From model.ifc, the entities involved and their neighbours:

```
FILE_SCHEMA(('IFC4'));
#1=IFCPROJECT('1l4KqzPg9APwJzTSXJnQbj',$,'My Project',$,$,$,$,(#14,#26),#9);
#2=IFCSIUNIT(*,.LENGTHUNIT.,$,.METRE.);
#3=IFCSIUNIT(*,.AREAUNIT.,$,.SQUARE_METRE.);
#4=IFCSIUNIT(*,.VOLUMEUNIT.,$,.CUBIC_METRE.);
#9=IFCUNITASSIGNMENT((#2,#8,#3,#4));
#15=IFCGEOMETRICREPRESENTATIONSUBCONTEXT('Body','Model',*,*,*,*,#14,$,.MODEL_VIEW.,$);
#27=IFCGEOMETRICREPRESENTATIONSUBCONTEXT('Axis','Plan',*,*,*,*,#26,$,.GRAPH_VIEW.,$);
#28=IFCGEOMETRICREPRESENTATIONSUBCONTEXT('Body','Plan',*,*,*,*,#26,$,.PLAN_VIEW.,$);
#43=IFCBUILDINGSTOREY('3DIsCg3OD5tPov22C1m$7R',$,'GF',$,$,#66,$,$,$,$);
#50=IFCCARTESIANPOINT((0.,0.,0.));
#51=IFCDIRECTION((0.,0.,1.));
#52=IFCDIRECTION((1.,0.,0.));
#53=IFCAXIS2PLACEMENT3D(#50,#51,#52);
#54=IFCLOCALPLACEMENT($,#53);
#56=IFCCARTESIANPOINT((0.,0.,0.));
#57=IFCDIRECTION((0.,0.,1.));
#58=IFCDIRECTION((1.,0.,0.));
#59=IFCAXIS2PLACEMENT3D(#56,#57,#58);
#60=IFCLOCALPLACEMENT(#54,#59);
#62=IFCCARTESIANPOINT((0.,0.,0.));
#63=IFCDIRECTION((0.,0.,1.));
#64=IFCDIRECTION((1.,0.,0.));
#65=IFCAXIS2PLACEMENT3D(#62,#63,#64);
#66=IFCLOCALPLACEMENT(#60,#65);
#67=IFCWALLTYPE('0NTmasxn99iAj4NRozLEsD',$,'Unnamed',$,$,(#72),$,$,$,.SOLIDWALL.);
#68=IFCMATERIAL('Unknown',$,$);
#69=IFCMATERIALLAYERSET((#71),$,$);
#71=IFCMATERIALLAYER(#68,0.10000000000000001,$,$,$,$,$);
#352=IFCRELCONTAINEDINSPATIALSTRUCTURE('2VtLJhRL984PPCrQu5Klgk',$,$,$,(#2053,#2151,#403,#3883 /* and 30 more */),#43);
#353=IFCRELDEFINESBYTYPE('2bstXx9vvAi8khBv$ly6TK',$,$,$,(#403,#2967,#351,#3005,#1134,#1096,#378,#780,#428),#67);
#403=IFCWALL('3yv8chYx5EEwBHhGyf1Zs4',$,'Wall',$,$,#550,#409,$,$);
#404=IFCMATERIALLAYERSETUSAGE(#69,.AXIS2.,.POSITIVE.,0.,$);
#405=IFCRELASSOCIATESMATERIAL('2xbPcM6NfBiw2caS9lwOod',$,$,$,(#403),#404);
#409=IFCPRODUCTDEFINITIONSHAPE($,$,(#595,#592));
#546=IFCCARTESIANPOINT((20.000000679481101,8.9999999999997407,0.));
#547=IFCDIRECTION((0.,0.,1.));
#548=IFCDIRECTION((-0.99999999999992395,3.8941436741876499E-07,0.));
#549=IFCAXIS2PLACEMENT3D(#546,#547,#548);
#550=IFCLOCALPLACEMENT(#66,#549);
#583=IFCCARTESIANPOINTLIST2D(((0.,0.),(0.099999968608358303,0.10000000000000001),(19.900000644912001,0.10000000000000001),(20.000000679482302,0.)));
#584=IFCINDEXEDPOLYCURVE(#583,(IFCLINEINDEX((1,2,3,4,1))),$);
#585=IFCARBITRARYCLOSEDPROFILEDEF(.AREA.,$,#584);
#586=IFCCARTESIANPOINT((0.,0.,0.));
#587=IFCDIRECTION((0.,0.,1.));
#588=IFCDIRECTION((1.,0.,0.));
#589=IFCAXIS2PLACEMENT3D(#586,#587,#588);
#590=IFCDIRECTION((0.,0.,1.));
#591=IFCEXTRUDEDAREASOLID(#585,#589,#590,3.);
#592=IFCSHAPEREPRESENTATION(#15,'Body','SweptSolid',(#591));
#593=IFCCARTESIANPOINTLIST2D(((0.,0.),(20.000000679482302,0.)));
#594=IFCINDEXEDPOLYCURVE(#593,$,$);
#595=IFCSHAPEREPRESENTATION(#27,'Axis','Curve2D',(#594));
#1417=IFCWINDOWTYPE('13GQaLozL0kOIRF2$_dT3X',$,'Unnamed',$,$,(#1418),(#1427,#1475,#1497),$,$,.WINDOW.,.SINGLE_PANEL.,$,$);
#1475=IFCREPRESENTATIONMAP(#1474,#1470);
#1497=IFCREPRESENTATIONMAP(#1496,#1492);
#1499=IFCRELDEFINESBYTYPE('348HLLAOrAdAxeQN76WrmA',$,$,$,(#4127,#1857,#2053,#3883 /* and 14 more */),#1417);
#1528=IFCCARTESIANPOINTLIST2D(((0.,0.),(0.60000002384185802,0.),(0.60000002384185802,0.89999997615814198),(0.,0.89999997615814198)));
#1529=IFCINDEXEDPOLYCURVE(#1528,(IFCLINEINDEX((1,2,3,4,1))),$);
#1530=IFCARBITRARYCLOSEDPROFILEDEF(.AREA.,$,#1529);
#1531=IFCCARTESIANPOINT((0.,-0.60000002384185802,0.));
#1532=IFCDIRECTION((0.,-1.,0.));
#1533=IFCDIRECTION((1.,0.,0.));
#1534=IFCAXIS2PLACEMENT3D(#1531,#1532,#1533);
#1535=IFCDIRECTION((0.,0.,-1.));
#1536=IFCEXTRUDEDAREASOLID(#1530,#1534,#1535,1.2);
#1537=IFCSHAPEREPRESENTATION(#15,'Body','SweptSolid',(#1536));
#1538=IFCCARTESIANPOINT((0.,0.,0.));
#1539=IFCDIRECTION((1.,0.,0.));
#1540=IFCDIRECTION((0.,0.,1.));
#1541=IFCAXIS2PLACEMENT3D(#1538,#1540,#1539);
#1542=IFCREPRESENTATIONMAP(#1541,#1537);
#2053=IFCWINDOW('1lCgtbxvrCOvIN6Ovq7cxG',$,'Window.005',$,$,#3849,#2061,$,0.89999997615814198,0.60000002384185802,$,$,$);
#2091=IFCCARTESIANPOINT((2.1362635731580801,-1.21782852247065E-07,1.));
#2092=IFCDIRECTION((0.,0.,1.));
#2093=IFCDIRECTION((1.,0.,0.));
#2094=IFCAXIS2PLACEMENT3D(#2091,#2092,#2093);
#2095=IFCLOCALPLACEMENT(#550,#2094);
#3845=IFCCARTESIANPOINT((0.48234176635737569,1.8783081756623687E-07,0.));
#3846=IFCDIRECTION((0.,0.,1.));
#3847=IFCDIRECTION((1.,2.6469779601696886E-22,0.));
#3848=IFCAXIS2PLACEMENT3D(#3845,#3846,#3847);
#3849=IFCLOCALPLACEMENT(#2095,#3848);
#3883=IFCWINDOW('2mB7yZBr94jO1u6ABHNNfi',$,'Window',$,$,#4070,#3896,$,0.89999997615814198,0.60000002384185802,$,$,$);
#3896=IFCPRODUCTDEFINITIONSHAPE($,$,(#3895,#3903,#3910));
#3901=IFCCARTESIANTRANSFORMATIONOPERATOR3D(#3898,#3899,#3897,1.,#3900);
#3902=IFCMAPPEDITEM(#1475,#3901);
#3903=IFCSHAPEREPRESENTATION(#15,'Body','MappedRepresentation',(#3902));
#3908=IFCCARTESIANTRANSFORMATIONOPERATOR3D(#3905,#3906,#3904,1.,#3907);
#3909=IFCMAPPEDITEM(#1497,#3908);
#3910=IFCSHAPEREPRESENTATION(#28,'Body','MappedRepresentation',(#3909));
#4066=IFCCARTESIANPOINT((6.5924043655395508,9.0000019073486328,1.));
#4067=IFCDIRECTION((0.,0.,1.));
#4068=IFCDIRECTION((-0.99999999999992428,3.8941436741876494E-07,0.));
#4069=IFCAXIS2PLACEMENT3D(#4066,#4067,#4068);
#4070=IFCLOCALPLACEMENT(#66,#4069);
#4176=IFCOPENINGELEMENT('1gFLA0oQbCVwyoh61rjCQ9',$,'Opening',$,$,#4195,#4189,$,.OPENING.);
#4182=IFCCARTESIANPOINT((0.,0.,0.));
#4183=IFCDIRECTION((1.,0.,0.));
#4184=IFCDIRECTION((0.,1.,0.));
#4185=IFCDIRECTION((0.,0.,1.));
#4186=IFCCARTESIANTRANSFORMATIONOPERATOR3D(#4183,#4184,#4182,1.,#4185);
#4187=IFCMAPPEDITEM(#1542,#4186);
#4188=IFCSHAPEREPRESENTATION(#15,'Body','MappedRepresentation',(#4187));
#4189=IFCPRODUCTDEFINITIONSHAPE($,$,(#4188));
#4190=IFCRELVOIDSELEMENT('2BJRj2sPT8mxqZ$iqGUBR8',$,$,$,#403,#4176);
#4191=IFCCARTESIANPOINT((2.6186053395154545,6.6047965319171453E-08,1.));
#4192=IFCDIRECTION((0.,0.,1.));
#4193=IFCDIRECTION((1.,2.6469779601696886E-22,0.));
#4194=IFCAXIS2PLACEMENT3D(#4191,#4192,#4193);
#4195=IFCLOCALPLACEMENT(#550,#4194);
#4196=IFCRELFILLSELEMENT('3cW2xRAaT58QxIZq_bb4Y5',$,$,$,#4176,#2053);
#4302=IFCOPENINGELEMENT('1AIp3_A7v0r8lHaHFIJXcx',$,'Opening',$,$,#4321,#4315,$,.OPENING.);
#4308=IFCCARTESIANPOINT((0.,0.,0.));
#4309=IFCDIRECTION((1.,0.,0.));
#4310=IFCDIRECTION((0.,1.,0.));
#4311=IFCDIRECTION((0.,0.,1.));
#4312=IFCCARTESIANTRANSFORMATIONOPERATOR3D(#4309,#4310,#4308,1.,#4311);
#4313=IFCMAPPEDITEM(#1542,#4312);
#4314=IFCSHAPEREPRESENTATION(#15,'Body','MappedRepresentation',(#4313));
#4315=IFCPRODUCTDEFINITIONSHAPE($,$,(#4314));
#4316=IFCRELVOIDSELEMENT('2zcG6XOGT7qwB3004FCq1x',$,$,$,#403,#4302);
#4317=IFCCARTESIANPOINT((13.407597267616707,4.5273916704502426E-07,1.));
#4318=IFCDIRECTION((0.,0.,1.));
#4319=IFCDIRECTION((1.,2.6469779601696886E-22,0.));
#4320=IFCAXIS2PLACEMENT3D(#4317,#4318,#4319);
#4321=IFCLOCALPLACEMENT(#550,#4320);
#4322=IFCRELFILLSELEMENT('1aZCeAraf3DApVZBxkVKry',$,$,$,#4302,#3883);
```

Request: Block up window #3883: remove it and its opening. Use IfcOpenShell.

```python
import ifcopenshell
import ifcopenshell.api.feature
import ifcopenshell.api.root
import ifcopenshell.geom
import ifcopenshell.util.shape

model = ifcopenshell.open("model.ifc")
settings = ifcopenshell.geom.settings()


def volume(element):
    """Net volume in cubic metres, openings subtracted."""
    shape = ifcopenshell.geom.create_shape(settings, element)
    return ifcopenshell.util.shape.get_volume(shape.geometry)


window = model.by_id(3883)
opening = window.FillsVoids[0].RelatingOpeningElement
wall = opening.VoidsElements[0].RelatingBuildingElement
before = volume(wall)

ifcopenshell.api.root.remove_product(model, product=window)
ifcopenshell.api.feature.remove_feature(model, feature=opening)

after = volume(wall)

print(f"wall volume {before:.3f} -> {after:.3f} m3")

model.write("model_updated.ifc")
```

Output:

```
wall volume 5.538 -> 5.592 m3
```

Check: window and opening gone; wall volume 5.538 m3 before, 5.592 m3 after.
